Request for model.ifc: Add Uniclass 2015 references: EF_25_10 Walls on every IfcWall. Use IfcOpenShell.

First a look at what the model holds.

```python
import ifcopenshell

model = ifcopenshell.open("model.ifc")
print(model.schema)
print("classifications:", [c.Name for c in model.by_type("IfcClassification")])
for ifc_class in ("IfcDoor", "IfcRoof", "IfcStair", "IfcWall", "IfcWindow"):
    print(ifc_class, len(model.by_type(ifc_class)))
```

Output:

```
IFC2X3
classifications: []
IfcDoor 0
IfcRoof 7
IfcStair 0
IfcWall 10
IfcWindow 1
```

```python
import ifcopenshell
import ifcopenshell.api.classification

model = ifcopenshell.open("model.ifc")

# IFC2X3 requires Source and Edition and has no link from the project to the system.
system = model.create_entity("IfcClassification", Source="NBS", Edition="2015", Name="Uniclass 2015")

codes = {
    "IfcWall": ("EF_25_10", "Walls"),
}
for ifc_class, (code, name) in codes.items():
    products = model.by_type(ifc_class)
    ifcopenshell.api.classification.add_reference(
        model, products=products, classification=system, identification=code, name=name
    )
    print(code, len(products))

model.write("model_edited.ifc")
```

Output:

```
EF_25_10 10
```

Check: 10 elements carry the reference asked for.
